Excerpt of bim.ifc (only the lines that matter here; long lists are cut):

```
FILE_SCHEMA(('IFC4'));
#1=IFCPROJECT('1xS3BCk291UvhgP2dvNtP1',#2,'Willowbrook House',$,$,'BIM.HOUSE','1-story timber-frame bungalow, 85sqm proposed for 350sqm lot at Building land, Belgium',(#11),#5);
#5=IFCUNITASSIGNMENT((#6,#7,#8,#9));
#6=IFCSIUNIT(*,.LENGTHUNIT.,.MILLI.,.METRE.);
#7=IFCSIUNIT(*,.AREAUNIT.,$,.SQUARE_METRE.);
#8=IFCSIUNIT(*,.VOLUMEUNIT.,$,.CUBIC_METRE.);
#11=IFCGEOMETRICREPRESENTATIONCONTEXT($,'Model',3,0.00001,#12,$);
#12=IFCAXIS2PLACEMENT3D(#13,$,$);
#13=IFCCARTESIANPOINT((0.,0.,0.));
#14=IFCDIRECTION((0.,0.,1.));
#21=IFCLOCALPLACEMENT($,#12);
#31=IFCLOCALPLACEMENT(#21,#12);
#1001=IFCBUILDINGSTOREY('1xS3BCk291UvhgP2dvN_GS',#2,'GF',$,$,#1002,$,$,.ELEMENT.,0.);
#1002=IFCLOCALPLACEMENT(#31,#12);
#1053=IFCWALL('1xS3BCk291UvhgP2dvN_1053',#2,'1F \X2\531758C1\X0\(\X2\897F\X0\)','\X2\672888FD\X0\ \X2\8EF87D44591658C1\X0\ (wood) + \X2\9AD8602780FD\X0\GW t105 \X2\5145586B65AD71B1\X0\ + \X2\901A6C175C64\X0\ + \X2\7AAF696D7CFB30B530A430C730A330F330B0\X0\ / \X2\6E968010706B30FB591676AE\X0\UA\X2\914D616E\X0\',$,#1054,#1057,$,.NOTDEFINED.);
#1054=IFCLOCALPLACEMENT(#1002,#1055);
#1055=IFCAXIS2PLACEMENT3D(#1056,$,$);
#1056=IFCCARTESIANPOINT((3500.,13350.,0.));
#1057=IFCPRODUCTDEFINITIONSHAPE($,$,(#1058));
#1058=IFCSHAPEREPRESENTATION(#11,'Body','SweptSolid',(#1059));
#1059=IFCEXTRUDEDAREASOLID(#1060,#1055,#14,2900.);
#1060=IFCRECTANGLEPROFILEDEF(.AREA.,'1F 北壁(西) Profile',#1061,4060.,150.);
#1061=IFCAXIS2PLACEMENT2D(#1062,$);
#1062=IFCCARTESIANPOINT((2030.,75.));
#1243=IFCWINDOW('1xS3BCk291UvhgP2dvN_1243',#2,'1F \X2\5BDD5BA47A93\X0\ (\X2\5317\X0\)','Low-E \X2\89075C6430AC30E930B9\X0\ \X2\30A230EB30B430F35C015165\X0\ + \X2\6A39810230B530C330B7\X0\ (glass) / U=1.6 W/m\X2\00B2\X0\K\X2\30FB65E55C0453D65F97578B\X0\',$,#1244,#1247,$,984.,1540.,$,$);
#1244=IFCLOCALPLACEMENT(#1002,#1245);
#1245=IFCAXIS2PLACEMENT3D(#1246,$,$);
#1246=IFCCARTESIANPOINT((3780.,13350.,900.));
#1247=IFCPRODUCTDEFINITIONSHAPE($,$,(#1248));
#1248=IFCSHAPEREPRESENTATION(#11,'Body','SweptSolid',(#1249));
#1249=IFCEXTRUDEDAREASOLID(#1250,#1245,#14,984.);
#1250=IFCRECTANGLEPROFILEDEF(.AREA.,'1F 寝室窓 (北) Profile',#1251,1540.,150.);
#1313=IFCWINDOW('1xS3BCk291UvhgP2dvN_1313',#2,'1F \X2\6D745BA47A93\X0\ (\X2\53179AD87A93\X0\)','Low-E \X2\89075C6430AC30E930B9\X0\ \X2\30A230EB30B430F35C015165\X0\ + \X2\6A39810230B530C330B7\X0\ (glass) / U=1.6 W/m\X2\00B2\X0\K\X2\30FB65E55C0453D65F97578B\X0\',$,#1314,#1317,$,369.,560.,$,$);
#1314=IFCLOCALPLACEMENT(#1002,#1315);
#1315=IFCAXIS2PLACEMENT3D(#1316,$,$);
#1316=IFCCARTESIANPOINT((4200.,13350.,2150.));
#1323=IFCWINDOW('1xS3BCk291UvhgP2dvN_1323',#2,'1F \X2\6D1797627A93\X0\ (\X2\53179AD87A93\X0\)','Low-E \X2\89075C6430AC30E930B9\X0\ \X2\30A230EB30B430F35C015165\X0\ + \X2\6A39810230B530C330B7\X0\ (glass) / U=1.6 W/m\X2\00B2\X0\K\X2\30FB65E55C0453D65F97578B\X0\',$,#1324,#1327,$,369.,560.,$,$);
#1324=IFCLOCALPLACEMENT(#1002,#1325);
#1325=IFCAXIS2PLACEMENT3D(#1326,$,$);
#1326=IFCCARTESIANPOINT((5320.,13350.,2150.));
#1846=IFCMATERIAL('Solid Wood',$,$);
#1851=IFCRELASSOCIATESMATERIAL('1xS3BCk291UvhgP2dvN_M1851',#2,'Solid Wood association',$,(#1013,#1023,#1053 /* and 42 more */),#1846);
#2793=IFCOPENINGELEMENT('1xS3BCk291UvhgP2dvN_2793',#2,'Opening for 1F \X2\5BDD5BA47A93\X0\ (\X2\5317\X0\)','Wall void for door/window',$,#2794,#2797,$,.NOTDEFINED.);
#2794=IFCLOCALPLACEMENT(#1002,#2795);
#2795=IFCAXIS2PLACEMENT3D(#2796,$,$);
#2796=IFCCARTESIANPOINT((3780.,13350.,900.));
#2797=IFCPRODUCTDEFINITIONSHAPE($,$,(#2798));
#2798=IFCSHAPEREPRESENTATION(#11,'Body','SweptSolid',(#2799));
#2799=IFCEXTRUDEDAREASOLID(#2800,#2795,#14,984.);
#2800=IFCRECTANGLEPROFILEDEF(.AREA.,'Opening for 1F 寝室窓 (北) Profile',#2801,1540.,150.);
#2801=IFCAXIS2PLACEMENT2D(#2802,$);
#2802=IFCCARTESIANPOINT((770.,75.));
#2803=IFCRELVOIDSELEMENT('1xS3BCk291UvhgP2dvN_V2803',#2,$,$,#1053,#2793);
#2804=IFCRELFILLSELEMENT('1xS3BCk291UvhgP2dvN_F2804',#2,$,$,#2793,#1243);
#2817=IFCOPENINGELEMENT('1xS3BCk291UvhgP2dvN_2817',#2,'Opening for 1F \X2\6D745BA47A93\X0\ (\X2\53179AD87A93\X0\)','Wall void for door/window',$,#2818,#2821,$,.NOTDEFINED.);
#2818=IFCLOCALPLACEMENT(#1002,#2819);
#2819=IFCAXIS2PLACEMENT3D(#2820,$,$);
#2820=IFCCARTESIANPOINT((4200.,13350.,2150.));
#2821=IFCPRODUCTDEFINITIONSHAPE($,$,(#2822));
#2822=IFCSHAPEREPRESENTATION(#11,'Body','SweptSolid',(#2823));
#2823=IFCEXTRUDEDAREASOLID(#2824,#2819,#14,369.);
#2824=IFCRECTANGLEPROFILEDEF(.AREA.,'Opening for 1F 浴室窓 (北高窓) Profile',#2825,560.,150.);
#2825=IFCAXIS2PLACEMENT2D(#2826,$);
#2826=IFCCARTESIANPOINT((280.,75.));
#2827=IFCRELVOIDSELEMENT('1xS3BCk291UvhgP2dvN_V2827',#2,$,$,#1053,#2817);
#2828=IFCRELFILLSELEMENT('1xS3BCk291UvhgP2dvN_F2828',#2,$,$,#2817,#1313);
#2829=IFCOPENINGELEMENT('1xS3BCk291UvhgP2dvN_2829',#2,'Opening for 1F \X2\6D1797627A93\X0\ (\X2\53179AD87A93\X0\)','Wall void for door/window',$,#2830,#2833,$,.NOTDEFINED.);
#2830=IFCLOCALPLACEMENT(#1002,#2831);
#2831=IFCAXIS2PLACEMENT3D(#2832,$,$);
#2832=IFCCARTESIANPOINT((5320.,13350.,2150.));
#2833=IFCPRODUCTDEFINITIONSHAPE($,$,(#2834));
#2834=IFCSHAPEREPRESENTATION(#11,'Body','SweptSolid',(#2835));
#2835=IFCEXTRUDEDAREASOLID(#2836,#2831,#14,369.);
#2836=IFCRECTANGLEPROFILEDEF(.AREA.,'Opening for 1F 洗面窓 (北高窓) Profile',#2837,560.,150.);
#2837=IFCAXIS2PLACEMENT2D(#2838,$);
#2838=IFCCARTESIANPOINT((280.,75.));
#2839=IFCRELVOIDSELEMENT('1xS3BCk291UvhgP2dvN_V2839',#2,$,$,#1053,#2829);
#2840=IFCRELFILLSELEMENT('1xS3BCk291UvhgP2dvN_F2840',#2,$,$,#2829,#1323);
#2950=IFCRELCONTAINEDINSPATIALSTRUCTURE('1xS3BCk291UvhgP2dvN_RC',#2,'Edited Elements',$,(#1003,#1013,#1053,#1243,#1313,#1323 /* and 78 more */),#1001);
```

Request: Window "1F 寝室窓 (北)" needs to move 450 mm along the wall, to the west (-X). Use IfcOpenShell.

```python
import ifcopenshell
import ifcopenshell.api.geometry
import ifcopenshell.util.placement
import ifcopenshell.util.unit

model = ifcopenshell.open("bim.ifc")
unit_scale = ifcopenshell.util.unit.calculate_unit_scale(model)

window = model.by_id(1243)
opening = window.FillsVoids[0].RelatingOpeningElement
wall = opening.VoidsElements[0].RelatingBuildingElement

wall_matrix = ifcopenshell.util.placement.get_local_placement(wall.ObjectPlacement)
shift = wall_matrix[:3, 0] * -0.45 / unit_scale
before = ifcopenshell.util.placement.get_local_placement(window.ObjectPlacement)[:3, 3].copy()

# The window is not placed relative to its opening, so move both.
for product in (opening, window):
    matrix = ifcopenshell.util.placement.get_local_placement(product.ObjectPlacement)
    matrix[:3, 3] += shift
    ifcopenshell.api.geometry.edit_object_placement(model, product=product, matrix=matrix, is_si=False)

after = ifcopenshell.util.placement.get_local_placement(window.ObjectPlacement)[:3, 3]
print("window moved by", (after - before).round(3) + 0.0)

model.write("bim_v2.ifc")
```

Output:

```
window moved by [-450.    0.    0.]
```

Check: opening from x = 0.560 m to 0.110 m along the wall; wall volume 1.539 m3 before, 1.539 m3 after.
